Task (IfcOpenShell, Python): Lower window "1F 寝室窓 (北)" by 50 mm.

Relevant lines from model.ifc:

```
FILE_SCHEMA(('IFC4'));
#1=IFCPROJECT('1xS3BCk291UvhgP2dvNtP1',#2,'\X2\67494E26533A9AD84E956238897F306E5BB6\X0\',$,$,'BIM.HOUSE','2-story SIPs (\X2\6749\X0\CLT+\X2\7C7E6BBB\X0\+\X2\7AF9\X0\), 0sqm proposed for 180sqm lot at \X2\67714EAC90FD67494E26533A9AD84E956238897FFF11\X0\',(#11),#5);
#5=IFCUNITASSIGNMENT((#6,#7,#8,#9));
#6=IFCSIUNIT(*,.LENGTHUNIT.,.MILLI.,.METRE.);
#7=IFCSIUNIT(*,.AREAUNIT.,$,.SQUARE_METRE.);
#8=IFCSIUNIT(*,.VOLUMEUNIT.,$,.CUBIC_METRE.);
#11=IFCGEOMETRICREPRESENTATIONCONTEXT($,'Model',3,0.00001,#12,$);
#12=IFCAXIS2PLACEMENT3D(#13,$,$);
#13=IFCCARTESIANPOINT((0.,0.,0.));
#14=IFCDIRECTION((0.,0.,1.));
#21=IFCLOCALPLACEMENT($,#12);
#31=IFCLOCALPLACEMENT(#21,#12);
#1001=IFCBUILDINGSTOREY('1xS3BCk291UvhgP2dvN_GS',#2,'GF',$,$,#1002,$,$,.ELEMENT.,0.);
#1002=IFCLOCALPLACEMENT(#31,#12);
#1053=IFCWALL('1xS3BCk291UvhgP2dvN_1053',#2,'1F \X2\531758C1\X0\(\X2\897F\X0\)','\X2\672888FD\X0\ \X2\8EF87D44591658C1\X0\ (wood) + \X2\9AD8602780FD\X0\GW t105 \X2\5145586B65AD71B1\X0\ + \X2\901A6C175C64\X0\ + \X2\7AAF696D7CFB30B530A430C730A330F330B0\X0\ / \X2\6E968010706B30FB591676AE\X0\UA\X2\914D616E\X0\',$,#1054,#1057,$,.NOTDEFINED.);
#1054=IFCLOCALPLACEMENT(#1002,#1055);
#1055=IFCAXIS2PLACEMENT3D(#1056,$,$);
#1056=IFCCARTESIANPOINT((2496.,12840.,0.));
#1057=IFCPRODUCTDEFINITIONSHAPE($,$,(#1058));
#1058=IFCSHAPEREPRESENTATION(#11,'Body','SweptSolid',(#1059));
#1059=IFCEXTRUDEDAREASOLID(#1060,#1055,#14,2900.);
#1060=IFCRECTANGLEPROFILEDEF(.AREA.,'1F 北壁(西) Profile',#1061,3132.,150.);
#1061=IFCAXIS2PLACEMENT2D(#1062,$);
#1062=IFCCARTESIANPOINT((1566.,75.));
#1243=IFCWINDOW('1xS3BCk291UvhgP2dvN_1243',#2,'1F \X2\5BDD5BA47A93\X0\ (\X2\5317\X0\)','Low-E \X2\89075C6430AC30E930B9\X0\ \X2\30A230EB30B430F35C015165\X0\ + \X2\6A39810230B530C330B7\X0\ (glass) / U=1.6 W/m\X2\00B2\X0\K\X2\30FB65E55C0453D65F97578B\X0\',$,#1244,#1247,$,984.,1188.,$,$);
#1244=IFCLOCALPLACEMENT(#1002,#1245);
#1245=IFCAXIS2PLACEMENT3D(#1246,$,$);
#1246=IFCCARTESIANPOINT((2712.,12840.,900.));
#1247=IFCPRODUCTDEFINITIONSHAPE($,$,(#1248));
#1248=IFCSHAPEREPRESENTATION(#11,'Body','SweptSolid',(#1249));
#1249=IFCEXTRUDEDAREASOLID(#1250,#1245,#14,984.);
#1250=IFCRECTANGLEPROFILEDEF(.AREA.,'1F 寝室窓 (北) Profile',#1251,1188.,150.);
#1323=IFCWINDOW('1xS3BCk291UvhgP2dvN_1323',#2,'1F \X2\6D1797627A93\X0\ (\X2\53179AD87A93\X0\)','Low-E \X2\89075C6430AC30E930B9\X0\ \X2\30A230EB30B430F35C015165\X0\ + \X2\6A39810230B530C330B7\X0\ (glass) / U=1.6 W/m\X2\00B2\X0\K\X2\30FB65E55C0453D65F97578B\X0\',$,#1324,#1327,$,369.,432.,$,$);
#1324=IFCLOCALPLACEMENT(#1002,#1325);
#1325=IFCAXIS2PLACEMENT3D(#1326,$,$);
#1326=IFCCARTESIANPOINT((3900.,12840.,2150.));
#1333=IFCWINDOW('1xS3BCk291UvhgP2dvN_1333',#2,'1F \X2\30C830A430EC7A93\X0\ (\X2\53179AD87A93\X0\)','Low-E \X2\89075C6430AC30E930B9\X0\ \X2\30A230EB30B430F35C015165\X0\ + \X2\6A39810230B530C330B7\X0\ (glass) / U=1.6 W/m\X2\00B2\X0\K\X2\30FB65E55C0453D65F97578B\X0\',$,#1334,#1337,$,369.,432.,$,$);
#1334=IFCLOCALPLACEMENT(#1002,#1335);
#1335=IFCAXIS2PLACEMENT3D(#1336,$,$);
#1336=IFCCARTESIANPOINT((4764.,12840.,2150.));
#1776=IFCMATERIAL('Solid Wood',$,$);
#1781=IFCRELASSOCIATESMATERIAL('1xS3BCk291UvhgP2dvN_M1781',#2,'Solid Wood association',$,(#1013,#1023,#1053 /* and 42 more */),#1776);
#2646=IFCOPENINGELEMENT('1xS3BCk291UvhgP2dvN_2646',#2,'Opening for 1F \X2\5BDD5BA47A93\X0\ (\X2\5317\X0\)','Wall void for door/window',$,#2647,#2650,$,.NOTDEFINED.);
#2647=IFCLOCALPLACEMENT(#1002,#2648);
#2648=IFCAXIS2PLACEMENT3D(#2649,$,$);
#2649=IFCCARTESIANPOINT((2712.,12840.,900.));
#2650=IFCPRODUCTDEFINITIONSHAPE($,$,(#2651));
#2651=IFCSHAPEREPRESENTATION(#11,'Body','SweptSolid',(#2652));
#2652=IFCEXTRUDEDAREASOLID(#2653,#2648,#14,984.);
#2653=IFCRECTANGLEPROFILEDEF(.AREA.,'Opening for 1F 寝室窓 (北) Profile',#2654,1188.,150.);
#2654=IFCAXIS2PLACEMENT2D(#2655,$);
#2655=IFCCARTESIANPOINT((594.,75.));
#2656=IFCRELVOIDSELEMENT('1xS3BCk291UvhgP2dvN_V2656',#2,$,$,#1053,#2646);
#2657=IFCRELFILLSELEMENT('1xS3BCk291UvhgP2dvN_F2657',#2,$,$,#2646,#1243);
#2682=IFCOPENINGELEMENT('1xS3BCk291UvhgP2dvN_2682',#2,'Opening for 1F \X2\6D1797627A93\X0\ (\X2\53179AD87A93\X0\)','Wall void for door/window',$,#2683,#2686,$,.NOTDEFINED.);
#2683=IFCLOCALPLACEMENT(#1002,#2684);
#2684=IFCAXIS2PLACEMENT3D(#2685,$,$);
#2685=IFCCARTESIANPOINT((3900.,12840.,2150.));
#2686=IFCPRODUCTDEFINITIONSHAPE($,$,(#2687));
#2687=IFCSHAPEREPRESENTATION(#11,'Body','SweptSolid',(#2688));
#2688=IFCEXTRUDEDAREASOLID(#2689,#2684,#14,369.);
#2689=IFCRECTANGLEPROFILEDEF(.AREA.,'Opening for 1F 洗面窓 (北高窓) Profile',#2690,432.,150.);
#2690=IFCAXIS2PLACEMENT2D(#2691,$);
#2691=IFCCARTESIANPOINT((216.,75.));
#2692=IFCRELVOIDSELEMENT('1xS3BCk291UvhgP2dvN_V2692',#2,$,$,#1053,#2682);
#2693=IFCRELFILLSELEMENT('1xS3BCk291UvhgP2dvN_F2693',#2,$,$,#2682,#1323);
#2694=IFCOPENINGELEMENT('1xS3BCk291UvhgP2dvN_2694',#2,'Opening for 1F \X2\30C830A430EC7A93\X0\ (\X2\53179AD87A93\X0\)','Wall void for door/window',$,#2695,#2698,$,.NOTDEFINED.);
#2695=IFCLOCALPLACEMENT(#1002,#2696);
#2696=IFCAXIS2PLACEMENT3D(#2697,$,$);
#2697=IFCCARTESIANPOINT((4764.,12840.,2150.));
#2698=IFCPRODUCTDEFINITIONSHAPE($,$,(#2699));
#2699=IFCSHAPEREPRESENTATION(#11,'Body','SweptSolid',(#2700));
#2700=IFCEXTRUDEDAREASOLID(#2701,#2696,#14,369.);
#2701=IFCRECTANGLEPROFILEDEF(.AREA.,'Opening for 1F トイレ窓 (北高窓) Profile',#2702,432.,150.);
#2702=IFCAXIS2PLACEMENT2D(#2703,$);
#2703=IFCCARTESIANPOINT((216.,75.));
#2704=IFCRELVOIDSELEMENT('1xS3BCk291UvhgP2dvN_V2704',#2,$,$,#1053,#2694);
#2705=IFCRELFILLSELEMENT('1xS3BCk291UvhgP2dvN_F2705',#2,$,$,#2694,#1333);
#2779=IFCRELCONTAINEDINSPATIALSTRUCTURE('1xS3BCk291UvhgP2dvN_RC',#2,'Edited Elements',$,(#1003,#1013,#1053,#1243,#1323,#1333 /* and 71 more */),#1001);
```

```python
import numpy as np
import ifcopenshell
import ifcopenshell.api.geometry
import ifcopenshell.util.placement
import ifcopenshell.util.unit

model = ifcopenshell.open("model.ifc")
unit_scale = ifcopenshell.util.unit.calculate_unit_scale(model)

window = model.by_id(1243)
opening = window.FillsVoids[0].RelatingOpeningElement
dz = -0.05 / unit_scale

shift = np.array([0.0, 0.0, dz])
# The window is not placed relative to its opening, so move both.
for product in (opening, window):
    matrix = ifcopenshell.util.placement.get_local_placement(product.ObjectPlacement)
    matrix[:3, 3] += shift
    ifcopenshell.api.geometry.edit_object_placement(model, product=product, matrix=matrix, is_si=False)

print(f"moved by {dz * unit_scale:+.3f} m")

model.write("model_updated.ifc")
```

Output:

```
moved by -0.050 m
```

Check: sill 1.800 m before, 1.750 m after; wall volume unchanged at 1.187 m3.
